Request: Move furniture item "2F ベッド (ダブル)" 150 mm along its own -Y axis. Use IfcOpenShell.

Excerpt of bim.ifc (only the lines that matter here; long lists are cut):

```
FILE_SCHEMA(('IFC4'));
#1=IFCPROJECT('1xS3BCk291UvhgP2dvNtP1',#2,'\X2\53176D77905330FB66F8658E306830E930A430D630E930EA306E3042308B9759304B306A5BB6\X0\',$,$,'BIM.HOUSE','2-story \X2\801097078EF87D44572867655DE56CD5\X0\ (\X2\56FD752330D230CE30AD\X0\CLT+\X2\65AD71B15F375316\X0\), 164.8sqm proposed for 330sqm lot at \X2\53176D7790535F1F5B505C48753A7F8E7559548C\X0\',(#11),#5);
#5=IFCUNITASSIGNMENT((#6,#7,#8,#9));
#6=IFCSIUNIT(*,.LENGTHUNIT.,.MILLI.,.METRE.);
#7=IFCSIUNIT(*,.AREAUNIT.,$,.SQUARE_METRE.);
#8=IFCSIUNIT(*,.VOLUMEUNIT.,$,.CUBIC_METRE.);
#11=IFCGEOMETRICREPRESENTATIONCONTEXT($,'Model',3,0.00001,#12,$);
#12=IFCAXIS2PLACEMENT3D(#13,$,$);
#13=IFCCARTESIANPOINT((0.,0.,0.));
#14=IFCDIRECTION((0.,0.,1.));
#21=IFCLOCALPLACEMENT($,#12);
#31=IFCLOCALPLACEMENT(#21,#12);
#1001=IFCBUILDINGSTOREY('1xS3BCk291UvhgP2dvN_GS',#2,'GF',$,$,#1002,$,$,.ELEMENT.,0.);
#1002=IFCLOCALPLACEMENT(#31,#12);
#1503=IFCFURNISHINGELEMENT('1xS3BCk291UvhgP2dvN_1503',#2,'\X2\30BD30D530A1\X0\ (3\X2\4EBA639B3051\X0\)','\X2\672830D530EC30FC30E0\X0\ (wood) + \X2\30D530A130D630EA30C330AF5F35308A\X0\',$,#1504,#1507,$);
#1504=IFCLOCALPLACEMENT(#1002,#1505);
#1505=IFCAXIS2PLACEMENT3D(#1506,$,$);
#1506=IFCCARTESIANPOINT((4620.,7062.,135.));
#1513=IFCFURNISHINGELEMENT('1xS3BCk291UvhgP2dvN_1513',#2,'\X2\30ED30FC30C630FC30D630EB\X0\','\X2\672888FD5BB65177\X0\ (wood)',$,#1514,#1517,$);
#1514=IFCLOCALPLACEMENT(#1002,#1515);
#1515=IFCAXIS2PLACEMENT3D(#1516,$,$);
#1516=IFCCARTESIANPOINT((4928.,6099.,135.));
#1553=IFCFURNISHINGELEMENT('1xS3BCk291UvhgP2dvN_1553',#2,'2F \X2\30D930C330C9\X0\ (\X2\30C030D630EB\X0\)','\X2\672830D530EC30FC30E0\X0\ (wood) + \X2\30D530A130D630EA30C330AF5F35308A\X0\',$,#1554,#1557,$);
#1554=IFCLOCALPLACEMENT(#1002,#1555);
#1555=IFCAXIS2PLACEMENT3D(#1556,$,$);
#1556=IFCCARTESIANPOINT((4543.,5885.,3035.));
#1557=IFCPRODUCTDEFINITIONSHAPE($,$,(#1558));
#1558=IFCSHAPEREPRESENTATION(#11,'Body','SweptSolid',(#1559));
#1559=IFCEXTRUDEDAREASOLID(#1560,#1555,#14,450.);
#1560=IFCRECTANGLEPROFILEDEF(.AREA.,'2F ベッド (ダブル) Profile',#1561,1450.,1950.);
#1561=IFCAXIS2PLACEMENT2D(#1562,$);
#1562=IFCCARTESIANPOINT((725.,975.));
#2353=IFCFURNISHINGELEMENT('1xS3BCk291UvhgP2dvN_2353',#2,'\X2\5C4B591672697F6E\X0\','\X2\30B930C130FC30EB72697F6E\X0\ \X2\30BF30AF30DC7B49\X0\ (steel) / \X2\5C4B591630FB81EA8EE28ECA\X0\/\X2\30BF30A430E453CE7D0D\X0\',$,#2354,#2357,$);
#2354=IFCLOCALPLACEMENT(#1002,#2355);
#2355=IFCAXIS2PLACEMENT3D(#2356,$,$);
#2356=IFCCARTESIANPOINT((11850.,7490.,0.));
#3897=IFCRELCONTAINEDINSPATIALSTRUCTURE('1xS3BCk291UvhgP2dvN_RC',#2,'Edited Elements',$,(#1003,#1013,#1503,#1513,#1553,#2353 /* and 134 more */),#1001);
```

```python
import ifcopenshell
import ifcopenshell.api.geometry
import ifcopenshell.util.placement

model = ifcopenshell.open("bim.ifc")

item = model.by_guid("1xS3BCk291UvhgP2dvN_1553")
matrix = ifcopenshell.util.placement.get_local_placement(item.ObjectPlacement)
matrix[:3, 3] -= matrix[:3, 1] * 150.0
ifcopenshell.api.geometry.edit_object_placement(model, product=item, matrix=matrix, is_si=False)

print(ifcopenshell.util.placement.get_local_placement(item.ObjectPlacement).round(3) + 0.0)

model.write("bim_updated.ifc")
```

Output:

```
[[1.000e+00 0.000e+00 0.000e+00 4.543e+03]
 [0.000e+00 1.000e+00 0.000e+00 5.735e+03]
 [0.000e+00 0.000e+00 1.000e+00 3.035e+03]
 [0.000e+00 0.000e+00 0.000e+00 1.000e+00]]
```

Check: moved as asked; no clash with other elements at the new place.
